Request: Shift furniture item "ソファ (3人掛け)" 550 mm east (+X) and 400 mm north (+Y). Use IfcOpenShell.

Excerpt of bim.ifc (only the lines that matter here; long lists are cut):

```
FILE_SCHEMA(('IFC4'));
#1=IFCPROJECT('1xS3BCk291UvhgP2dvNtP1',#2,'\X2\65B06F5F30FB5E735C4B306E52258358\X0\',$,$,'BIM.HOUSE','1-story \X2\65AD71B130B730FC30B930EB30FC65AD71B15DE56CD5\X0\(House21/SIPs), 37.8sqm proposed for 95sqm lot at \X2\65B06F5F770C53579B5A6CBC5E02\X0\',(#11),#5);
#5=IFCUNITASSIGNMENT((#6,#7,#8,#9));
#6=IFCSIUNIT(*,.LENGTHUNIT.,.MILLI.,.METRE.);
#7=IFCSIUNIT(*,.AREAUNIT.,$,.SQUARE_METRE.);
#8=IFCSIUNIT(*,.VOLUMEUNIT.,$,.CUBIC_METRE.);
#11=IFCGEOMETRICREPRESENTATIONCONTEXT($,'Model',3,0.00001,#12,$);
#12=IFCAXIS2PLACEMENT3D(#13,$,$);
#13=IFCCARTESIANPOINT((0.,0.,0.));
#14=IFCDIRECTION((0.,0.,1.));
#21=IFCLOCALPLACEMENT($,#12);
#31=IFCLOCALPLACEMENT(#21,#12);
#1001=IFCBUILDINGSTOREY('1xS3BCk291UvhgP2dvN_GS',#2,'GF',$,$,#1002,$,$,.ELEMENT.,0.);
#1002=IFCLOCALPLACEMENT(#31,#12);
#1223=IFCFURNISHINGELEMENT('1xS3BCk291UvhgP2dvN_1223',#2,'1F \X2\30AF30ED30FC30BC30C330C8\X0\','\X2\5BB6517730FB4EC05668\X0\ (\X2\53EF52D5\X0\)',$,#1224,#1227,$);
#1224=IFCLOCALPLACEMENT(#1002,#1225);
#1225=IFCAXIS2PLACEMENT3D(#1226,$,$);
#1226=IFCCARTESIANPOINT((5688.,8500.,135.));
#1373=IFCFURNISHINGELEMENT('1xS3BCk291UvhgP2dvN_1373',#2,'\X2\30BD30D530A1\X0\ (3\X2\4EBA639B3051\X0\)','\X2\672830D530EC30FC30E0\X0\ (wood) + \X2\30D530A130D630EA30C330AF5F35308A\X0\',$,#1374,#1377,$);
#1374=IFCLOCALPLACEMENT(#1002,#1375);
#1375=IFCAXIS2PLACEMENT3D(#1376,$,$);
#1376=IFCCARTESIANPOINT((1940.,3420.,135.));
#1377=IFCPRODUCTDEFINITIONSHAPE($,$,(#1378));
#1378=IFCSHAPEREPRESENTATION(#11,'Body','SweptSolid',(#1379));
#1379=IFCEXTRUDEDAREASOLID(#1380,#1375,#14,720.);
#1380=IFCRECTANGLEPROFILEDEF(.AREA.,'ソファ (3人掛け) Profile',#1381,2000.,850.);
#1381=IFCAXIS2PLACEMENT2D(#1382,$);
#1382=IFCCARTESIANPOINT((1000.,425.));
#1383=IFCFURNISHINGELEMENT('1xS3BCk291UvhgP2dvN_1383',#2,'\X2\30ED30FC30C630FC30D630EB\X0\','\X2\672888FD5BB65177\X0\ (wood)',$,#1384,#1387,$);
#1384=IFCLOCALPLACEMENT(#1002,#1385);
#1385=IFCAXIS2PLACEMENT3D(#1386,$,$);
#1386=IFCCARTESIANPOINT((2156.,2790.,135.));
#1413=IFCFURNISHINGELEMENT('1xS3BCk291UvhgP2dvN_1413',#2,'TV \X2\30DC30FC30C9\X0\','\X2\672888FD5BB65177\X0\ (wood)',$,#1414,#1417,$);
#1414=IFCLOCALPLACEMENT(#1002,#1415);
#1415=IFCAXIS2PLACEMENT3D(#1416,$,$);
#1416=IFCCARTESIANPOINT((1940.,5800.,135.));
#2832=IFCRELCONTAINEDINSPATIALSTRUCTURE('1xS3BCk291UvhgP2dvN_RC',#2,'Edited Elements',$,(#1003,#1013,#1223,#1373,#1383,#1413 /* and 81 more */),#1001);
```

```python
import ifcopenshell
import ifcopenshell.api.geometry
import ifcopenshell.util.placement

model = ifcopenshell.open("bim.ifc")

item = model.by_guid("1xS3BCk291UvhgP2dvN_1373")
matrix = ifcopenshell.util.placement.get_local_placement(item.ObjectPlacement)
matrix[0, 3] += 550.0
matrix[1, 3] += 400.0
ifcopenshell.api.geometry.edit_object_placement(model, product=item, matrix=matrix, is_si=False)

print(ifcopenshell.util.placement.get_local_placement(item.ObjectPlacement).round(3) + 0.0)

model.write("bim_rev.ifc")
```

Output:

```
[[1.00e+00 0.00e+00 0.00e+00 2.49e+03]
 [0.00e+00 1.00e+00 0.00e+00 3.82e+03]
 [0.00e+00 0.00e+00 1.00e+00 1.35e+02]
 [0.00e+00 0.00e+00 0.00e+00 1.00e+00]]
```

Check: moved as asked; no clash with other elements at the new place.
